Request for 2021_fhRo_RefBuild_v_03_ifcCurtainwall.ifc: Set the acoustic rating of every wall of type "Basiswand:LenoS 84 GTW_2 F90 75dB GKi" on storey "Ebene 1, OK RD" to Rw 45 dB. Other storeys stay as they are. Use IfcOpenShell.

First a look at what the model holds.

```python
import ifcopenshell
import ifcopenshell.util.element

model = ifcopenshell.open("2021_fhRo_RefBuild_v_03_ifcCurtainwall.ifc")
print(model.schema)
storey = next(s for s in model.by_type("IfcBuildingStorey") if s.Name == "Ebene 1, OK RD")
walls = [e for e in ifcopenshell.util.element.get_decomposition(storey) if e.is_a("IfcWall")]
seen = {}
for e in walls:
    element_type = ifcopenshell.util.element.get_type(e)
    key = (element_type.Name if element_type != e and element_type else None, ifcopenshell.util.element.get_pset(e, "Pset_WallCommon", "AcousticRating"))
    seen[key] = seen.get(key, 0) + 1
for (name, value), count in sorted(seen.items(), key=str):
    print(count, "x", name, "|", value)
```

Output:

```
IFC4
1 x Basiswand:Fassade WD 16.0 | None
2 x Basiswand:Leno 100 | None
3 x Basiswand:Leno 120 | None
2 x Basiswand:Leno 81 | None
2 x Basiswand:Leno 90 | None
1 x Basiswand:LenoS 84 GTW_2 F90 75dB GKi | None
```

```python
import ifcopenshell
import ifcopenshell.api.pset
import ifcopenshell.util.element

model = ifcopenshell.open("2021_fhRo_RefBuild_v_03_ifcCurtainwall.ifc")

storey = next(s for s in model.by_type("IfcBuildingStorey") if s.Name == "Ebene 1, OK RD")
walls = [e for e in ifcopenshell.util.element.get_decomposition(storey) if e.is_a("IfcWall")]

count = 0
for e in walls:
    element_type = ifcopenshell.util.element.get_type(e)
    if element_type in (None, e) or element_type.Name != "Basiswand:LenoS 84 GTW_2 F90 75dB GKi":
        continue
    # add_pset returns the element's existing set when there is one.
    pset = ifcopenshell.api.pset.add_pset(model, product=e, name="Pset_WallCommon")
    ifcopenshell.api.pset.edit_pset(model, pset=pset, properties={"AcousticRating": "Rw 45 dB"})
    count += 1

print(count, "walls updated")

model.write("2021_fhRo_RefBuild_v_03_ifcCurtainwall-out.ifc")
```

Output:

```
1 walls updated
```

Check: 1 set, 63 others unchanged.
